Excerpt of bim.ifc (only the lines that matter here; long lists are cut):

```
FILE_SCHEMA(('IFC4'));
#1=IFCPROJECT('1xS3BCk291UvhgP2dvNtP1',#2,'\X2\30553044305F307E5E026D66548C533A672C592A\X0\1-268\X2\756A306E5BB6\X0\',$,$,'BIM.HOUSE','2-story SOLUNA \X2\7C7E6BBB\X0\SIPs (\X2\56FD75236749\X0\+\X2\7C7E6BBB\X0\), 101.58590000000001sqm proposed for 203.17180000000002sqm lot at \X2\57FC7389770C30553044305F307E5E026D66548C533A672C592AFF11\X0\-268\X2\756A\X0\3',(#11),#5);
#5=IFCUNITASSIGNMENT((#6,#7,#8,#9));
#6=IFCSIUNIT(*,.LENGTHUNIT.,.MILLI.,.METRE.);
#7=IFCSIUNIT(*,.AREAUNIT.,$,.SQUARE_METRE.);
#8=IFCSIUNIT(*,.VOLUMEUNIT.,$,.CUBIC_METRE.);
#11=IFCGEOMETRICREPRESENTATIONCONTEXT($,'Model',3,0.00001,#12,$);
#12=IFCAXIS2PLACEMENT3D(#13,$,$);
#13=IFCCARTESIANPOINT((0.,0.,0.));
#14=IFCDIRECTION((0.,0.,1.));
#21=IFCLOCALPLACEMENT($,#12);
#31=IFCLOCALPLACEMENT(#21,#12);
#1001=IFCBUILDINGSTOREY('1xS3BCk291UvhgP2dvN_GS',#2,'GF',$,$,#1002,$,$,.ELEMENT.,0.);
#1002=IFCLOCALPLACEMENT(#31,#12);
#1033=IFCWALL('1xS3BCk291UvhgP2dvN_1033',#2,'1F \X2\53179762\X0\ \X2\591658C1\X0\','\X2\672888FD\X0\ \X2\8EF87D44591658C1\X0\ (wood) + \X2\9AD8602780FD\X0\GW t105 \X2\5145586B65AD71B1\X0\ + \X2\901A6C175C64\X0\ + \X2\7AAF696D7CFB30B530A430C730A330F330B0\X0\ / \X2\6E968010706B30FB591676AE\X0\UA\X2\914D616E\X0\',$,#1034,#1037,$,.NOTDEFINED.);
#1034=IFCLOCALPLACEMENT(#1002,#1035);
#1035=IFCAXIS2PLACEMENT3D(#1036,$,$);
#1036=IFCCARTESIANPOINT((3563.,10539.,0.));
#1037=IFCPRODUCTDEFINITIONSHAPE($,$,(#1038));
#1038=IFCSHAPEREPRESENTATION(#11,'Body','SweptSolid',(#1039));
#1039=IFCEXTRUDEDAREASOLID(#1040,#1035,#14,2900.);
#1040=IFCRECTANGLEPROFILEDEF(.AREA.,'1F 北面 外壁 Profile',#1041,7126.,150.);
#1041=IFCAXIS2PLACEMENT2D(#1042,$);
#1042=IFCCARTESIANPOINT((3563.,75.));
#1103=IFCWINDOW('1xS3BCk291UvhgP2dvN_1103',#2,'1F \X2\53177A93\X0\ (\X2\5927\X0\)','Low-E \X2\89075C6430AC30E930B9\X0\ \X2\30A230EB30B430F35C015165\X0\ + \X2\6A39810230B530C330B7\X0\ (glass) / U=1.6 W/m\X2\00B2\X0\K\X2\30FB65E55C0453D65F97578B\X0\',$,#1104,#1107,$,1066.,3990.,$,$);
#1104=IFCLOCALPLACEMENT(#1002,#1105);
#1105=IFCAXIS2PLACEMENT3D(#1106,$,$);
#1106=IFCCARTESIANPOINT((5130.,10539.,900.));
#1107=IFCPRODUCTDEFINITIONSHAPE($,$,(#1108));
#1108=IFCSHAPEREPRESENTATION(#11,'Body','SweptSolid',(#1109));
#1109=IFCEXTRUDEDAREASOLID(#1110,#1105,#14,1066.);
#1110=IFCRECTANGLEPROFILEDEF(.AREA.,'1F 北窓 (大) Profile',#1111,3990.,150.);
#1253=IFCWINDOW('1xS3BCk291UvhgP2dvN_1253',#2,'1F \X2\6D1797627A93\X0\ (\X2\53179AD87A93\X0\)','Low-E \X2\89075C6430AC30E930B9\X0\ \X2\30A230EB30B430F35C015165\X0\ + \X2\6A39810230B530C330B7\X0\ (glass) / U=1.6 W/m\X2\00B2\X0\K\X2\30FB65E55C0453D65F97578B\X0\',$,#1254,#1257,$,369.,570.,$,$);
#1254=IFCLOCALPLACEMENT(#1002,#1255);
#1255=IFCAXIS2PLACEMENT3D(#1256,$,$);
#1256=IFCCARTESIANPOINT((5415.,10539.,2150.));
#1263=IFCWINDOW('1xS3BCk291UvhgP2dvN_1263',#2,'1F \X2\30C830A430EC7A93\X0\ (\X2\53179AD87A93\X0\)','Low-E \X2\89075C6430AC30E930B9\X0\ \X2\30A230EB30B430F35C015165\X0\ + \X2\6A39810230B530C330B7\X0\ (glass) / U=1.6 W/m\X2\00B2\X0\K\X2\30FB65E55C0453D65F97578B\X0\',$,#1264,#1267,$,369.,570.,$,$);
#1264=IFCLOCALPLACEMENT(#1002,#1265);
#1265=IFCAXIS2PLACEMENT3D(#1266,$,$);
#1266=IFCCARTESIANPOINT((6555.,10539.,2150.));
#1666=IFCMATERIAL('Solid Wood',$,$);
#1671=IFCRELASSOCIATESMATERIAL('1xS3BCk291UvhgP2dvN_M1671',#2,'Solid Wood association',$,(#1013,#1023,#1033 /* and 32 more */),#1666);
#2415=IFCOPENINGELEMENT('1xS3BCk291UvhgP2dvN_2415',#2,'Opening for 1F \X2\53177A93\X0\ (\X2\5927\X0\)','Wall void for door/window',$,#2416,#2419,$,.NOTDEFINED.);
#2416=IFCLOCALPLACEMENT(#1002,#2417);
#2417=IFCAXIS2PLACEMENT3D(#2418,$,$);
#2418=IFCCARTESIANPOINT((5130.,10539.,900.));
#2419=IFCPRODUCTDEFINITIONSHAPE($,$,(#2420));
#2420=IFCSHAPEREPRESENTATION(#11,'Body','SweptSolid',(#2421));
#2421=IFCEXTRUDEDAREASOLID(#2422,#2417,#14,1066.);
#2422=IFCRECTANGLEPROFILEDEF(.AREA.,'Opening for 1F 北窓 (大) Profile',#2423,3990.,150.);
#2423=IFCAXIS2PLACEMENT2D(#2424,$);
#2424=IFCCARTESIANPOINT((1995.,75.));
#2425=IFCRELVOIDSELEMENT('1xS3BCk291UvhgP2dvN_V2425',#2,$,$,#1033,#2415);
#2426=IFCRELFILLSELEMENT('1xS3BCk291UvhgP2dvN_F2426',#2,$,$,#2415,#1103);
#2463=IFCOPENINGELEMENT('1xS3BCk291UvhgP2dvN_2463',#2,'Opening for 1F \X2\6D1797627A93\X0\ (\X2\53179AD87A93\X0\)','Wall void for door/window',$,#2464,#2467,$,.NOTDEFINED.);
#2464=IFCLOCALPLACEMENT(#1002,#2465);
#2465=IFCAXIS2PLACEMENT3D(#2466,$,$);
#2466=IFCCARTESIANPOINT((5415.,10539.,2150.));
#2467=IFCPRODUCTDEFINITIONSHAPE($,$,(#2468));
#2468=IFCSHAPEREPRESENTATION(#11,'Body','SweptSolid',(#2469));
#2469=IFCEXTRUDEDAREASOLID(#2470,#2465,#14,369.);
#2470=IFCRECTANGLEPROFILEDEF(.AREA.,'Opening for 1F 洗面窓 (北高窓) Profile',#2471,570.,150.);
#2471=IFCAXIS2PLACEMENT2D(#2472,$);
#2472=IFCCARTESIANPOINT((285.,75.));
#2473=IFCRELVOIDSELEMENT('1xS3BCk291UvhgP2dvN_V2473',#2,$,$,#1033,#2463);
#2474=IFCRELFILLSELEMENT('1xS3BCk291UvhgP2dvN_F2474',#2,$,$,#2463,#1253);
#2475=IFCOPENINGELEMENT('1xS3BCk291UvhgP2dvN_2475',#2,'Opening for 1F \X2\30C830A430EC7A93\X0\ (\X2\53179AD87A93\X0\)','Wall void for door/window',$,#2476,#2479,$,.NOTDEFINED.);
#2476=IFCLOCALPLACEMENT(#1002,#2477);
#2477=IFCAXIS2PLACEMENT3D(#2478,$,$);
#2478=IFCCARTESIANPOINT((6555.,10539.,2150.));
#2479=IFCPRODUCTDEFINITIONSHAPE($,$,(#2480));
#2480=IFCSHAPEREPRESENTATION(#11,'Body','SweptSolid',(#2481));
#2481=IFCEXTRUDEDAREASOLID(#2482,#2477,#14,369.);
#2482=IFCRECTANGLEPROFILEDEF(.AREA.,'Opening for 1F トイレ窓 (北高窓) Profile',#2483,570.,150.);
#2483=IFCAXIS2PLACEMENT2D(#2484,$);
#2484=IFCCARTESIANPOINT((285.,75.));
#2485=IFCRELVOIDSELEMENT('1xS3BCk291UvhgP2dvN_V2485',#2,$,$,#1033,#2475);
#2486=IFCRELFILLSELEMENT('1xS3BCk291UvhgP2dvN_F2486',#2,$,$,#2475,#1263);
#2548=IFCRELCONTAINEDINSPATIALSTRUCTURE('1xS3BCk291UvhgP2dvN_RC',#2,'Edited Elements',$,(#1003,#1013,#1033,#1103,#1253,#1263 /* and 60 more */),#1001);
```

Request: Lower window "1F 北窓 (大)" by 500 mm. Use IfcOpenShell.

```python
import numpy as np
import ifcopenshell
import ifcopenshell.api.geometry
import ifcopenshell.util.placement
import ifcopenshell.util.unit

model = ifcopenshell.open("bim.ifc")
unit_scale = ifcopenshell.util.unit.calculate_unit_scale(model)

window = model.by_id(1103)
opening = window.FillsVoids[0].RelatingOpeningElement
dz = -500.0

shift = np.array([0.0, 0.0, dz])
# The window is not placed relative to its opening, so move both.
for product in (opening, window):
    matrix = ifcopenshell.util.placement.get_local_placement(product.ObjectPlacement)
    matrix[:3, 3] += shift
    ifcopenshell.api.geometry.edit_object_placement(model, product=product, matrix=matrix, is_si=False)

print(f"moved by {dz * unit_scale:+.3f} m")

model.write("bim_rev.ifc")
```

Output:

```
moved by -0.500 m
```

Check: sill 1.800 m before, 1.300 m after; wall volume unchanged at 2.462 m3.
